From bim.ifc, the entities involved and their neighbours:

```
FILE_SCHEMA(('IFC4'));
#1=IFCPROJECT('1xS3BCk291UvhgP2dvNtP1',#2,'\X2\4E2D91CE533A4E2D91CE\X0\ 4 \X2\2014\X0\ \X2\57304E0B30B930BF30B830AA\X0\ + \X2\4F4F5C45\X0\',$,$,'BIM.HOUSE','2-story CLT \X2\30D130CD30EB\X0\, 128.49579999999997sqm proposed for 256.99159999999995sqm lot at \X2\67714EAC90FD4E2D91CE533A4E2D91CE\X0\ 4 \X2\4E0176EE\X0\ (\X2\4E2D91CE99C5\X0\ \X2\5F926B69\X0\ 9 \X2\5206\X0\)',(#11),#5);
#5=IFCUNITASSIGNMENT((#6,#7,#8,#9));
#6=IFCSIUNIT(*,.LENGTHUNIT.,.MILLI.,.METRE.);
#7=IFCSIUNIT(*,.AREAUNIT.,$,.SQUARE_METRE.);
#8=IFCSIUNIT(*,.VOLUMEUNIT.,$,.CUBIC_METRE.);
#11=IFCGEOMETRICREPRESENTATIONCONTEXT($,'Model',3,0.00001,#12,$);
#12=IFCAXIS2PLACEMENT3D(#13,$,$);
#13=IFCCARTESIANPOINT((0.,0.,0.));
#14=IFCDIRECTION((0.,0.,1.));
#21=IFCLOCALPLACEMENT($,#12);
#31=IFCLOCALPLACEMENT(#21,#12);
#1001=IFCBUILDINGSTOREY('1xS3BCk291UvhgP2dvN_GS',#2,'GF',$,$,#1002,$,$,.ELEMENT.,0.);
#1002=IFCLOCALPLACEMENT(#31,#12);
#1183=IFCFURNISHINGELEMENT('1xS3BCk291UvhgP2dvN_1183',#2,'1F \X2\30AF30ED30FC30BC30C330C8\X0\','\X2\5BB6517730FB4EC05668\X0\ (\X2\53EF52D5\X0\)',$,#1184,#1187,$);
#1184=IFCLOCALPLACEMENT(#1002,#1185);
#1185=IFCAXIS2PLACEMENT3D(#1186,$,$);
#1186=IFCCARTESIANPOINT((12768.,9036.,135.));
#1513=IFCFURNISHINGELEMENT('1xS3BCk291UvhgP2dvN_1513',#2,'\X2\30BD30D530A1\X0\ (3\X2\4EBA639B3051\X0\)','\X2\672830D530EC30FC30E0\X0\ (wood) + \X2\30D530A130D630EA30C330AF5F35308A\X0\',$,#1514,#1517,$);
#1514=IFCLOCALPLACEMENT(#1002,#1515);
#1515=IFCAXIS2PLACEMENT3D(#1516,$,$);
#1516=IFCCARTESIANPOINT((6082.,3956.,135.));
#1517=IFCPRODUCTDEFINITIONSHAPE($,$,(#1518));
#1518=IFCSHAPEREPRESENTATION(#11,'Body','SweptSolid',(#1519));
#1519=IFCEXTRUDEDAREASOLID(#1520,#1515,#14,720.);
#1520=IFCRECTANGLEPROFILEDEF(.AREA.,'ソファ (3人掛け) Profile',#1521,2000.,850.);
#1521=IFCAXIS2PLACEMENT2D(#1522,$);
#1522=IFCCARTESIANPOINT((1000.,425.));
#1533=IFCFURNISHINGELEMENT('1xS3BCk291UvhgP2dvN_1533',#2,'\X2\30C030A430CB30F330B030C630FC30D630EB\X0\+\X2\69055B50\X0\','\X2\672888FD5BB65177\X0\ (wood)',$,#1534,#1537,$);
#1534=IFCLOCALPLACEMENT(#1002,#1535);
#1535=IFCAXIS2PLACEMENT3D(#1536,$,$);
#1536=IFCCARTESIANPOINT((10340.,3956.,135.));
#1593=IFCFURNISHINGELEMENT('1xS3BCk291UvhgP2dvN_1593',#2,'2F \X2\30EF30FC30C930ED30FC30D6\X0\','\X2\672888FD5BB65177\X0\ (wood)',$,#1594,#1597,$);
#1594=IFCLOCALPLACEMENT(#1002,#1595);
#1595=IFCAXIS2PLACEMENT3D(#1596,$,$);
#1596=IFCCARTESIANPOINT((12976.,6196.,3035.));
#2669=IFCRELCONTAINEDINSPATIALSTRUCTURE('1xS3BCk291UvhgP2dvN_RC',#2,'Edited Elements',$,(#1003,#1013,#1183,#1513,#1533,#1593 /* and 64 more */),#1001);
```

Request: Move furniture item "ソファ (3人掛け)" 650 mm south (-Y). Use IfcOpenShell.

```python
import ifcopenshell
import ifcopenshell.api.geometry
import ifcopenshell.util.placement

model = ifcopenshell.open("bim.ifc")

item = model.by_guid("1xS3BCk291UvhgP2dvN_1513")
matrix = ifcopenshell.util.placement.get_local_placement(item.ObjectPlacement)
matrix[1, 3] -= 650.0
ifcopenshell.api.geometry.edit_object_placement(model, product=item, matrix=matrix, is_si=False)

print(ifcopenshell.util.placement.get_local_placement(item.ObjectPlacement).round(3) + 0.0)

model.write("bim_edited.ifc")
```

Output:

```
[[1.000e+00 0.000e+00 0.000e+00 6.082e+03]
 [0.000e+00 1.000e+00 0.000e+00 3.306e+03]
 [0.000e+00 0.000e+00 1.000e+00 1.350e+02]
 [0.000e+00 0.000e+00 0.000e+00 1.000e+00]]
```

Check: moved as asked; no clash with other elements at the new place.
